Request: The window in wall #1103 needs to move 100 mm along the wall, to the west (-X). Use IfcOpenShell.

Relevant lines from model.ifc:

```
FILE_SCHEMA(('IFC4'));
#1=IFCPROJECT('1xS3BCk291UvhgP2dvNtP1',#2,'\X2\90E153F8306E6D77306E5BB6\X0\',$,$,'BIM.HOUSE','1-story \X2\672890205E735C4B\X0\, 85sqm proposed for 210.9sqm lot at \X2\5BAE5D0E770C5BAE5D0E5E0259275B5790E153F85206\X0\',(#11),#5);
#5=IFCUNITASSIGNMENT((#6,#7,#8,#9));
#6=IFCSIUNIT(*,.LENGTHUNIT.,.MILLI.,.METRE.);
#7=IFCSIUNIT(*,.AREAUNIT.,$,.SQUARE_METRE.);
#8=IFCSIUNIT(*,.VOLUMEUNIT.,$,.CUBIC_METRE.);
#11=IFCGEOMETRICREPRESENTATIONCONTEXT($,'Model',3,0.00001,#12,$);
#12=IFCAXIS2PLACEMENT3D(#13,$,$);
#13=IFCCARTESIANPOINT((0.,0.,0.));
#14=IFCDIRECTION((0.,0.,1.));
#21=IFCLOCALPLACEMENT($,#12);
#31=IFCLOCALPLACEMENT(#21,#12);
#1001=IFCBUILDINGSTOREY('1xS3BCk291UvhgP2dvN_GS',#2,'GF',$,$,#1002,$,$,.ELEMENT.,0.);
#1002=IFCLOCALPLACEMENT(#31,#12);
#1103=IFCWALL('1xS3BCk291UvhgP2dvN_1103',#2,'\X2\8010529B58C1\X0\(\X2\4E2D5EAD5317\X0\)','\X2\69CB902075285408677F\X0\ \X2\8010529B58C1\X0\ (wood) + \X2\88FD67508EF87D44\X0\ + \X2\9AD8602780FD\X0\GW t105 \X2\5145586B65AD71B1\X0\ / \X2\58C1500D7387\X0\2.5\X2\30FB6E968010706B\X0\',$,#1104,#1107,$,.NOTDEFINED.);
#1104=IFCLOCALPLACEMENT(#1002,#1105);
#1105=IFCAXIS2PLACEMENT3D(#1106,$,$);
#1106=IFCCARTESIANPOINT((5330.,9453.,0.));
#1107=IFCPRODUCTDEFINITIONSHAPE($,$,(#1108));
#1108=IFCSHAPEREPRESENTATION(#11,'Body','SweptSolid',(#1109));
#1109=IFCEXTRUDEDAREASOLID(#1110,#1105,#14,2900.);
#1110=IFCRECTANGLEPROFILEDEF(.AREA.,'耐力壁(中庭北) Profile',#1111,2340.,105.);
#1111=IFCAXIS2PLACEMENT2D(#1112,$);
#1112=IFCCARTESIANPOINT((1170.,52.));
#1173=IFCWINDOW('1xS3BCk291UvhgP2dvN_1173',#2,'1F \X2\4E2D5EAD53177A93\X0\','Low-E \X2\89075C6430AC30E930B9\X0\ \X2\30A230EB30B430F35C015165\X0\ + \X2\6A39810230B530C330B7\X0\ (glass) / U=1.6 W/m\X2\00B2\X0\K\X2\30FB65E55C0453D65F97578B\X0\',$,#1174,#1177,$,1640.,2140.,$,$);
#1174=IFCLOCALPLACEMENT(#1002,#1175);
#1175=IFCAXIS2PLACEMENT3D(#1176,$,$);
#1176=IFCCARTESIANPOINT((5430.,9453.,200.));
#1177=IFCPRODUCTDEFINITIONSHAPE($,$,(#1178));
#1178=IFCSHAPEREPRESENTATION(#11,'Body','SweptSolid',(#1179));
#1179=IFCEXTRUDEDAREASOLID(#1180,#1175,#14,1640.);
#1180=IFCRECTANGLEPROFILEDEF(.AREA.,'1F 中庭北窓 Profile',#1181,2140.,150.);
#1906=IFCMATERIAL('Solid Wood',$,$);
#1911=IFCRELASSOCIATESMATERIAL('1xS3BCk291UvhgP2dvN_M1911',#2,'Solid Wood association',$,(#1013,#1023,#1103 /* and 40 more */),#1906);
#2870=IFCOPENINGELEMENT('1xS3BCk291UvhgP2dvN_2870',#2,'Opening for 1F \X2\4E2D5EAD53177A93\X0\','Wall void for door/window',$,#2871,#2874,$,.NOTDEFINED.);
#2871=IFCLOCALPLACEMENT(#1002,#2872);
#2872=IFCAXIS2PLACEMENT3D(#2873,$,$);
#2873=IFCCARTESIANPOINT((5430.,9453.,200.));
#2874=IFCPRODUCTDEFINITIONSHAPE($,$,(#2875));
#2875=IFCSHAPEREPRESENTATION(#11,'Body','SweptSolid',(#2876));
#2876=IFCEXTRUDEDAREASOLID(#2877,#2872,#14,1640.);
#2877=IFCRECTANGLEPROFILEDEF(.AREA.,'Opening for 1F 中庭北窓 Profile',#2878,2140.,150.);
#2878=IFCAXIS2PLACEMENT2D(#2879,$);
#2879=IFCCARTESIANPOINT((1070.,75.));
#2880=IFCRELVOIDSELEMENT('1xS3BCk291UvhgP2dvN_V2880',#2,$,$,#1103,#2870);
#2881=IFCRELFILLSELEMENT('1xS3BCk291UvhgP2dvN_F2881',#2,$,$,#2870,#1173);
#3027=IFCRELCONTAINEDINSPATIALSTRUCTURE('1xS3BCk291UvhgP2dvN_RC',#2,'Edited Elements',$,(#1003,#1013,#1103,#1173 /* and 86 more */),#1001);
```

```python
import ifcopenshell
import ifcopenshell.api.geometry
import ifcopenshell.util.placement
import ifcopenshell.util.unit

model = ifcopenshell.open("model.ifc")
unit_scale = ifcopenshell.util.unit.calculate_unit_scale(model)

window = model.by_guid("1xS3BCk291UvhgP2dvN_1173")
opening = window.FillsVoids[0].RelatingOpeningElement
wall = opening.VoidsElements[0].RelatingBuildingElement

wall_matrix = ifcopenshell.util.placement.get_local_placement(wall.ObjectPlacement)
shift = wall_matrix[:3, 0] * -0.1 / unit_scale
before = ifcopenshell.util.placement.get_local_placement(window.ObjectPlacement)[:3, 3].copy()

# The window is not placed relative to its opening, so move both.
for product in (opening, window):
    matrix = ifcopenshell.util.placement.get_local_placement(product.ObjectPlacement)
    matrix[:3, 3] += shift
    ifcopenshell.api.geometry.edit_object_placement(model, product=product, matrix=matrix, is_si=False)

after = ifcopenshell.util.placement.get_local_placement(window.ObjectPlacement)[:3, 3]
print("window moved by", (after - before).round(3) + 0.0)

model.write("model_v2.ifc")
```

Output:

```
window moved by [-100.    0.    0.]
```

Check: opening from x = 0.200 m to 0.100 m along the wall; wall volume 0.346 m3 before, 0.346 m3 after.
